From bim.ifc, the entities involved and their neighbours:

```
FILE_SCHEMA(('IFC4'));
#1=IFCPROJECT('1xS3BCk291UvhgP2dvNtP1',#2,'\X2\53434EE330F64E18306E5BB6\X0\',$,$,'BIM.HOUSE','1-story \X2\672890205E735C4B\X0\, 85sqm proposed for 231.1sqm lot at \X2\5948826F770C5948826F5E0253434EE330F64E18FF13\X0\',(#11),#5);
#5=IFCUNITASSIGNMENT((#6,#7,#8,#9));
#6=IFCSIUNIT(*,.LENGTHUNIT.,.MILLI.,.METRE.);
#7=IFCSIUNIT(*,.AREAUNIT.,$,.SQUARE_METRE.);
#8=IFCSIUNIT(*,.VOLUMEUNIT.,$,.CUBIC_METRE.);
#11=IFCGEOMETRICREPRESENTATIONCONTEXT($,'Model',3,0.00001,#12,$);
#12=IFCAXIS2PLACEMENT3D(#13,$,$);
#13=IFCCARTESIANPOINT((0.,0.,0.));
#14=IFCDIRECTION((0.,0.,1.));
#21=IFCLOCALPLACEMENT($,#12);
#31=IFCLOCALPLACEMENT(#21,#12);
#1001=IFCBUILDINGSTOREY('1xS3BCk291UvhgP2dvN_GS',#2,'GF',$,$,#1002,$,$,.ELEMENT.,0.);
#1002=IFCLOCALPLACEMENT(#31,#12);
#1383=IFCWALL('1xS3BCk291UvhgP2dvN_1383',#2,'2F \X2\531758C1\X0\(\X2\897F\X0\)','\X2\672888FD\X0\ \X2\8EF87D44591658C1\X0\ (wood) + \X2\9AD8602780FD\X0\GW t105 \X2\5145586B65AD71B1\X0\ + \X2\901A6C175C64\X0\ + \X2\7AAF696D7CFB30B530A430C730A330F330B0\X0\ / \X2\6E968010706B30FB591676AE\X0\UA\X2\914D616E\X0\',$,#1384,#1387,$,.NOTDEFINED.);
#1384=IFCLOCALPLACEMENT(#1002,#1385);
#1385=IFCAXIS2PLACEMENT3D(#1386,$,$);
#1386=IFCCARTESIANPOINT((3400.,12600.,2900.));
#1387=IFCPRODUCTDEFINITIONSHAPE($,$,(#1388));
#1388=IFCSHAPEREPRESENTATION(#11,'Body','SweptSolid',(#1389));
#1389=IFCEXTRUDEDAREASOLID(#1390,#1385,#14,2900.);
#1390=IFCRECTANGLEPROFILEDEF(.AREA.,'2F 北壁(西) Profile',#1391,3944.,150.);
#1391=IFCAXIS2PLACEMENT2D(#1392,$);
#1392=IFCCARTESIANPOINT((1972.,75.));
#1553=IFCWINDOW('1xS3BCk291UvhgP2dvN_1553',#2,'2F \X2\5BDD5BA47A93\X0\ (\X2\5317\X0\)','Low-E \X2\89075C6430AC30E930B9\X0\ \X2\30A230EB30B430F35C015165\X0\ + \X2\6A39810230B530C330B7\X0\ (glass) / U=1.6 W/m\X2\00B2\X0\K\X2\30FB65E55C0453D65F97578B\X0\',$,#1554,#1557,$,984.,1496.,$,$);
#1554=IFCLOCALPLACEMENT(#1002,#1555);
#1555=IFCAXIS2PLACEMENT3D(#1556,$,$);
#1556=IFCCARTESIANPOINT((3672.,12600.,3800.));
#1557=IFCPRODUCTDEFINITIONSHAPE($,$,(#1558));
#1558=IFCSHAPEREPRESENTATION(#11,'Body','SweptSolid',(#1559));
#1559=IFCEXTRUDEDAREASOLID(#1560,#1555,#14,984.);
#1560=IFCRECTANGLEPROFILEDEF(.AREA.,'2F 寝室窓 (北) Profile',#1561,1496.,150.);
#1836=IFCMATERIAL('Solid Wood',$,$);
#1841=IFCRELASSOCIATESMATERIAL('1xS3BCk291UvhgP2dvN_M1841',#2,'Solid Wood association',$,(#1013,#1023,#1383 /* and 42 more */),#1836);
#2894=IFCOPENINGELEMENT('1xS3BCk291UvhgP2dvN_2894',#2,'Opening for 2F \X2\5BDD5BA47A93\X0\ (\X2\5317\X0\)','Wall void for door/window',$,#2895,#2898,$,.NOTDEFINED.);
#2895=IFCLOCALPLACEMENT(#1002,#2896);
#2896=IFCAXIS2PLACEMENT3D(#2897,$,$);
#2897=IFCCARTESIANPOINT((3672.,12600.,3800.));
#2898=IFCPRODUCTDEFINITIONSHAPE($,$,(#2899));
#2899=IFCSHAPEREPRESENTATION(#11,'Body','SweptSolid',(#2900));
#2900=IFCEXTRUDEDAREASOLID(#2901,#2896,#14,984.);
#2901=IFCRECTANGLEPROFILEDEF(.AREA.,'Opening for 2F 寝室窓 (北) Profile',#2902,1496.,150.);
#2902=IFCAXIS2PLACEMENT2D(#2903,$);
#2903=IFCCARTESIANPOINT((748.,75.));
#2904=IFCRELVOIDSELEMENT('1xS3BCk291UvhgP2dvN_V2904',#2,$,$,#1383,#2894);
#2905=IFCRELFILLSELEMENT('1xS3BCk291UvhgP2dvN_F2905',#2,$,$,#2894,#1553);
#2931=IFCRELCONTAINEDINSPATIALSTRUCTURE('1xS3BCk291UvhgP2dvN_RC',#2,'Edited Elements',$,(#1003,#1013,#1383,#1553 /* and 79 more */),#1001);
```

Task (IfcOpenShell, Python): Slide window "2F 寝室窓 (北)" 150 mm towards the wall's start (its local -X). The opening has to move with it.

```python
import ifcopenshell
import ifcopenshell.api.geometry
import ifcopenshell.util.placement

model = ifcopenshell.open("bim.ifc")

window = model.by_id(1553)
opening = window.FillsVoids[0].RelatingOpeningElement
wall = opening.VoidsElements[0].RelatingBuildingElement

wall_matrix = ifcopenshell.util.placement.get_local_placement(wall.ObjectPlacement)
shift = wall_matrix[:3, 0] * -150.0
before = ifcopenshell.util.placement.get_local_placement(window.ObjectPlacement)[:3, 3].copy()

# The window is not placed relative to its opening, so move both.
for product in (opening, window):
    matrix = ifcopenshell.util.placement.get_local_placement(product.ObjectPlacement)
    matrix[:3, 3] += shift
    ifcopenshell.api.geometry.edit_object_placement(model, product=product, matrix=matrix, is_si=False)

after = ifcopenshell.util.placement.get_local_placement(window.ObjectPlacement)[:3, 3]
print("window moved by", (after - before).round(3) + 0.0)

model.write("bim_updated.ifc")
```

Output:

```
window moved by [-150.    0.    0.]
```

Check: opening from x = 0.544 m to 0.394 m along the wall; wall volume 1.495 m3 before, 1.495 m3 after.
